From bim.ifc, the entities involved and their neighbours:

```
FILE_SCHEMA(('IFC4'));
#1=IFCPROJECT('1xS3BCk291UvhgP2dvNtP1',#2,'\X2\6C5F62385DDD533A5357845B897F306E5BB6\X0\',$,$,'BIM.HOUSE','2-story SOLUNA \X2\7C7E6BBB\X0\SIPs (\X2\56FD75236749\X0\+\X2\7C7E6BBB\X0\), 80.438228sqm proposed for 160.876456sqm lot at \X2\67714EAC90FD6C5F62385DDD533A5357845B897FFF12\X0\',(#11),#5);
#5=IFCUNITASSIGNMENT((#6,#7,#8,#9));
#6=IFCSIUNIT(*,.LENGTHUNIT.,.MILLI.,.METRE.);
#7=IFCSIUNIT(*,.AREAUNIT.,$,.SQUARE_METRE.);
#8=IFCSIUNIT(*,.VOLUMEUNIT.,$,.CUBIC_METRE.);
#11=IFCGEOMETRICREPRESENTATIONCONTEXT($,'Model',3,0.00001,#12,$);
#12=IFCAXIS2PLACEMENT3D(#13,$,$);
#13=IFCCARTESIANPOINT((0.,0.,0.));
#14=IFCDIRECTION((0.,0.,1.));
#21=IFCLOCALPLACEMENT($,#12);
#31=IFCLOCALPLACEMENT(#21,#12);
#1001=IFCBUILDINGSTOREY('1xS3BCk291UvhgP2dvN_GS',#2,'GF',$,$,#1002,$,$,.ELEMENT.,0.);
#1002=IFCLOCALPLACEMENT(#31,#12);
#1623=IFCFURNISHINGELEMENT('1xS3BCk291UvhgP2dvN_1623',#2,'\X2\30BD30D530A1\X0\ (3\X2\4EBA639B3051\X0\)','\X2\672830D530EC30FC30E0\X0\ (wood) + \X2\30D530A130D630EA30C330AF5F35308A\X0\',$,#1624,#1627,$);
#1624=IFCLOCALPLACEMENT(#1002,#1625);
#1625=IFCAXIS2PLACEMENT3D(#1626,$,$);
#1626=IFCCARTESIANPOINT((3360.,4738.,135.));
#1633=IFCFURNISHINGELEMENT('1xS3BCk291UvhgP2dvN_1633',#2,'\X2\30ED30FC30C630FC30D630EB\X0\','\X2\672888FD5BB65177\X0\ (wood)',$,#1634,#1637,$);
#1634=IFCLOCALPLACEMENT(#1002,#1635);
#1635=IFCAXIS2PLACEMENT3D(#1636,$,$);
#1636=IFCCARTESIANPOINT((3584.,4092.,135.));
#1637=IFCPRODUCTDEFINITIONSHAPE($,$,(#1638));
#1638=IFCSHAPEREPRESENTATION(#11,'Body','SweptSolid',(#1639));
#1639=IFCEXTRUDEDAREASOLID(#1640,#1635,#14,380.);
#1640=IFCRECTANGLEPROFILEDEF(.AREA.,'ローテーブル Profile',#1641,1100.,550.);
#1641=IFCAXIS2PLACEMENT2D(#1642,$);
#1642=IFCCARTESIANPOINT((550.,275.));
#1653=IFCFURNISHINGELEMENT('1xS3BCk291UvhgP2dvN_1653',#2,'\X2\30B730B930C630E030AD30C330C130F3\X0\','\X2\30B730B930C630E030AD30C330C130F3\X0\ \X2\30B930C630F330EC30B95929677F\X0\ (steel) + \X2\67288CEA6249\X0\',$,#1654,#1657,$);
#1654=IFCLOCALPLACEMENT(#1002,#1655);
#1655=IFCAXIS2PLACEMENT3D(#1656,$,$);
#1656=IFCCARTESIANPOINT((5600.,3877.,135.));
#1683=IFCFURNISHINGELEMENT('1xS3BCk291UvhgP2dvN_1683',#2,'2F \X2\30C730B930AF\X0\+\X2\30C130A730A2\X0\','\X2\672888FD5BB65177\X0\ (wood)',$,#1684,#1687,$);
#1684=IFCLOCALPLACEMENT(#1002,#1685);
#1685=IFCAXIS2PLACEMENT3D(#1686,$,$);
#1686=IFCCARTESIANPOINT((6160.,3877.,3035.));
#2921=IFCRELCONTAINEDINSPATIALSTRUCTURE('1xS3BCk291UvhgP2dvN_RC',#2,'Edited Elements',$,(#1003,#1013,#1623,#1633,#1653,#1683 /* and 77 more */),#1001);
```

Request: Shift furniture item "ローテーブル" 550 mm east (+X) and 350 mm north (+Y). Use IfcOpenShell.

```python
import ifcopenshell
import ifcopenshell.api.geometry
import ifcopenshell.util.placement
import ifcopenshell.util.unit

model = ifcopenshell.open("bim.ifc")
unit_scale = ifcopenshell.util.unit.calculate_unit_scale(model)

item = model.by_guid("1xS3BCk291UvhgP2dvN_1633")
matrix = ifcopenshell.util.placement.get_local_placement(item.ObjectPlacement)
matrix[0, 3] += 0.55 / unit_scale
matrix[1, 3] += 0.35 / unit_scale
ifcopenshell.api.geometry.edit_object_placement(model, product=item, matrix=matrix, is_si=False)

print(ifcopenshell.util.placement.get_local_placement(item.ObjectPlacement).round(3) + 0.0)

model.write("bim_edited.ifc")
```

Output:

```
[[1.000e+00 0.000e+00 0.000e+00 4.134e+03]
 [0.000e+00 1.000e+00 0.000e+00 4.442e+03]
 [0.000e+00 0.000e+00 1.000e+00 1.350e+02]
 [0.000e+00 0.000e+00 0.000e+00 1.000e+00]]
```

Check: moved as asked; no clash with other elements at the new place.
